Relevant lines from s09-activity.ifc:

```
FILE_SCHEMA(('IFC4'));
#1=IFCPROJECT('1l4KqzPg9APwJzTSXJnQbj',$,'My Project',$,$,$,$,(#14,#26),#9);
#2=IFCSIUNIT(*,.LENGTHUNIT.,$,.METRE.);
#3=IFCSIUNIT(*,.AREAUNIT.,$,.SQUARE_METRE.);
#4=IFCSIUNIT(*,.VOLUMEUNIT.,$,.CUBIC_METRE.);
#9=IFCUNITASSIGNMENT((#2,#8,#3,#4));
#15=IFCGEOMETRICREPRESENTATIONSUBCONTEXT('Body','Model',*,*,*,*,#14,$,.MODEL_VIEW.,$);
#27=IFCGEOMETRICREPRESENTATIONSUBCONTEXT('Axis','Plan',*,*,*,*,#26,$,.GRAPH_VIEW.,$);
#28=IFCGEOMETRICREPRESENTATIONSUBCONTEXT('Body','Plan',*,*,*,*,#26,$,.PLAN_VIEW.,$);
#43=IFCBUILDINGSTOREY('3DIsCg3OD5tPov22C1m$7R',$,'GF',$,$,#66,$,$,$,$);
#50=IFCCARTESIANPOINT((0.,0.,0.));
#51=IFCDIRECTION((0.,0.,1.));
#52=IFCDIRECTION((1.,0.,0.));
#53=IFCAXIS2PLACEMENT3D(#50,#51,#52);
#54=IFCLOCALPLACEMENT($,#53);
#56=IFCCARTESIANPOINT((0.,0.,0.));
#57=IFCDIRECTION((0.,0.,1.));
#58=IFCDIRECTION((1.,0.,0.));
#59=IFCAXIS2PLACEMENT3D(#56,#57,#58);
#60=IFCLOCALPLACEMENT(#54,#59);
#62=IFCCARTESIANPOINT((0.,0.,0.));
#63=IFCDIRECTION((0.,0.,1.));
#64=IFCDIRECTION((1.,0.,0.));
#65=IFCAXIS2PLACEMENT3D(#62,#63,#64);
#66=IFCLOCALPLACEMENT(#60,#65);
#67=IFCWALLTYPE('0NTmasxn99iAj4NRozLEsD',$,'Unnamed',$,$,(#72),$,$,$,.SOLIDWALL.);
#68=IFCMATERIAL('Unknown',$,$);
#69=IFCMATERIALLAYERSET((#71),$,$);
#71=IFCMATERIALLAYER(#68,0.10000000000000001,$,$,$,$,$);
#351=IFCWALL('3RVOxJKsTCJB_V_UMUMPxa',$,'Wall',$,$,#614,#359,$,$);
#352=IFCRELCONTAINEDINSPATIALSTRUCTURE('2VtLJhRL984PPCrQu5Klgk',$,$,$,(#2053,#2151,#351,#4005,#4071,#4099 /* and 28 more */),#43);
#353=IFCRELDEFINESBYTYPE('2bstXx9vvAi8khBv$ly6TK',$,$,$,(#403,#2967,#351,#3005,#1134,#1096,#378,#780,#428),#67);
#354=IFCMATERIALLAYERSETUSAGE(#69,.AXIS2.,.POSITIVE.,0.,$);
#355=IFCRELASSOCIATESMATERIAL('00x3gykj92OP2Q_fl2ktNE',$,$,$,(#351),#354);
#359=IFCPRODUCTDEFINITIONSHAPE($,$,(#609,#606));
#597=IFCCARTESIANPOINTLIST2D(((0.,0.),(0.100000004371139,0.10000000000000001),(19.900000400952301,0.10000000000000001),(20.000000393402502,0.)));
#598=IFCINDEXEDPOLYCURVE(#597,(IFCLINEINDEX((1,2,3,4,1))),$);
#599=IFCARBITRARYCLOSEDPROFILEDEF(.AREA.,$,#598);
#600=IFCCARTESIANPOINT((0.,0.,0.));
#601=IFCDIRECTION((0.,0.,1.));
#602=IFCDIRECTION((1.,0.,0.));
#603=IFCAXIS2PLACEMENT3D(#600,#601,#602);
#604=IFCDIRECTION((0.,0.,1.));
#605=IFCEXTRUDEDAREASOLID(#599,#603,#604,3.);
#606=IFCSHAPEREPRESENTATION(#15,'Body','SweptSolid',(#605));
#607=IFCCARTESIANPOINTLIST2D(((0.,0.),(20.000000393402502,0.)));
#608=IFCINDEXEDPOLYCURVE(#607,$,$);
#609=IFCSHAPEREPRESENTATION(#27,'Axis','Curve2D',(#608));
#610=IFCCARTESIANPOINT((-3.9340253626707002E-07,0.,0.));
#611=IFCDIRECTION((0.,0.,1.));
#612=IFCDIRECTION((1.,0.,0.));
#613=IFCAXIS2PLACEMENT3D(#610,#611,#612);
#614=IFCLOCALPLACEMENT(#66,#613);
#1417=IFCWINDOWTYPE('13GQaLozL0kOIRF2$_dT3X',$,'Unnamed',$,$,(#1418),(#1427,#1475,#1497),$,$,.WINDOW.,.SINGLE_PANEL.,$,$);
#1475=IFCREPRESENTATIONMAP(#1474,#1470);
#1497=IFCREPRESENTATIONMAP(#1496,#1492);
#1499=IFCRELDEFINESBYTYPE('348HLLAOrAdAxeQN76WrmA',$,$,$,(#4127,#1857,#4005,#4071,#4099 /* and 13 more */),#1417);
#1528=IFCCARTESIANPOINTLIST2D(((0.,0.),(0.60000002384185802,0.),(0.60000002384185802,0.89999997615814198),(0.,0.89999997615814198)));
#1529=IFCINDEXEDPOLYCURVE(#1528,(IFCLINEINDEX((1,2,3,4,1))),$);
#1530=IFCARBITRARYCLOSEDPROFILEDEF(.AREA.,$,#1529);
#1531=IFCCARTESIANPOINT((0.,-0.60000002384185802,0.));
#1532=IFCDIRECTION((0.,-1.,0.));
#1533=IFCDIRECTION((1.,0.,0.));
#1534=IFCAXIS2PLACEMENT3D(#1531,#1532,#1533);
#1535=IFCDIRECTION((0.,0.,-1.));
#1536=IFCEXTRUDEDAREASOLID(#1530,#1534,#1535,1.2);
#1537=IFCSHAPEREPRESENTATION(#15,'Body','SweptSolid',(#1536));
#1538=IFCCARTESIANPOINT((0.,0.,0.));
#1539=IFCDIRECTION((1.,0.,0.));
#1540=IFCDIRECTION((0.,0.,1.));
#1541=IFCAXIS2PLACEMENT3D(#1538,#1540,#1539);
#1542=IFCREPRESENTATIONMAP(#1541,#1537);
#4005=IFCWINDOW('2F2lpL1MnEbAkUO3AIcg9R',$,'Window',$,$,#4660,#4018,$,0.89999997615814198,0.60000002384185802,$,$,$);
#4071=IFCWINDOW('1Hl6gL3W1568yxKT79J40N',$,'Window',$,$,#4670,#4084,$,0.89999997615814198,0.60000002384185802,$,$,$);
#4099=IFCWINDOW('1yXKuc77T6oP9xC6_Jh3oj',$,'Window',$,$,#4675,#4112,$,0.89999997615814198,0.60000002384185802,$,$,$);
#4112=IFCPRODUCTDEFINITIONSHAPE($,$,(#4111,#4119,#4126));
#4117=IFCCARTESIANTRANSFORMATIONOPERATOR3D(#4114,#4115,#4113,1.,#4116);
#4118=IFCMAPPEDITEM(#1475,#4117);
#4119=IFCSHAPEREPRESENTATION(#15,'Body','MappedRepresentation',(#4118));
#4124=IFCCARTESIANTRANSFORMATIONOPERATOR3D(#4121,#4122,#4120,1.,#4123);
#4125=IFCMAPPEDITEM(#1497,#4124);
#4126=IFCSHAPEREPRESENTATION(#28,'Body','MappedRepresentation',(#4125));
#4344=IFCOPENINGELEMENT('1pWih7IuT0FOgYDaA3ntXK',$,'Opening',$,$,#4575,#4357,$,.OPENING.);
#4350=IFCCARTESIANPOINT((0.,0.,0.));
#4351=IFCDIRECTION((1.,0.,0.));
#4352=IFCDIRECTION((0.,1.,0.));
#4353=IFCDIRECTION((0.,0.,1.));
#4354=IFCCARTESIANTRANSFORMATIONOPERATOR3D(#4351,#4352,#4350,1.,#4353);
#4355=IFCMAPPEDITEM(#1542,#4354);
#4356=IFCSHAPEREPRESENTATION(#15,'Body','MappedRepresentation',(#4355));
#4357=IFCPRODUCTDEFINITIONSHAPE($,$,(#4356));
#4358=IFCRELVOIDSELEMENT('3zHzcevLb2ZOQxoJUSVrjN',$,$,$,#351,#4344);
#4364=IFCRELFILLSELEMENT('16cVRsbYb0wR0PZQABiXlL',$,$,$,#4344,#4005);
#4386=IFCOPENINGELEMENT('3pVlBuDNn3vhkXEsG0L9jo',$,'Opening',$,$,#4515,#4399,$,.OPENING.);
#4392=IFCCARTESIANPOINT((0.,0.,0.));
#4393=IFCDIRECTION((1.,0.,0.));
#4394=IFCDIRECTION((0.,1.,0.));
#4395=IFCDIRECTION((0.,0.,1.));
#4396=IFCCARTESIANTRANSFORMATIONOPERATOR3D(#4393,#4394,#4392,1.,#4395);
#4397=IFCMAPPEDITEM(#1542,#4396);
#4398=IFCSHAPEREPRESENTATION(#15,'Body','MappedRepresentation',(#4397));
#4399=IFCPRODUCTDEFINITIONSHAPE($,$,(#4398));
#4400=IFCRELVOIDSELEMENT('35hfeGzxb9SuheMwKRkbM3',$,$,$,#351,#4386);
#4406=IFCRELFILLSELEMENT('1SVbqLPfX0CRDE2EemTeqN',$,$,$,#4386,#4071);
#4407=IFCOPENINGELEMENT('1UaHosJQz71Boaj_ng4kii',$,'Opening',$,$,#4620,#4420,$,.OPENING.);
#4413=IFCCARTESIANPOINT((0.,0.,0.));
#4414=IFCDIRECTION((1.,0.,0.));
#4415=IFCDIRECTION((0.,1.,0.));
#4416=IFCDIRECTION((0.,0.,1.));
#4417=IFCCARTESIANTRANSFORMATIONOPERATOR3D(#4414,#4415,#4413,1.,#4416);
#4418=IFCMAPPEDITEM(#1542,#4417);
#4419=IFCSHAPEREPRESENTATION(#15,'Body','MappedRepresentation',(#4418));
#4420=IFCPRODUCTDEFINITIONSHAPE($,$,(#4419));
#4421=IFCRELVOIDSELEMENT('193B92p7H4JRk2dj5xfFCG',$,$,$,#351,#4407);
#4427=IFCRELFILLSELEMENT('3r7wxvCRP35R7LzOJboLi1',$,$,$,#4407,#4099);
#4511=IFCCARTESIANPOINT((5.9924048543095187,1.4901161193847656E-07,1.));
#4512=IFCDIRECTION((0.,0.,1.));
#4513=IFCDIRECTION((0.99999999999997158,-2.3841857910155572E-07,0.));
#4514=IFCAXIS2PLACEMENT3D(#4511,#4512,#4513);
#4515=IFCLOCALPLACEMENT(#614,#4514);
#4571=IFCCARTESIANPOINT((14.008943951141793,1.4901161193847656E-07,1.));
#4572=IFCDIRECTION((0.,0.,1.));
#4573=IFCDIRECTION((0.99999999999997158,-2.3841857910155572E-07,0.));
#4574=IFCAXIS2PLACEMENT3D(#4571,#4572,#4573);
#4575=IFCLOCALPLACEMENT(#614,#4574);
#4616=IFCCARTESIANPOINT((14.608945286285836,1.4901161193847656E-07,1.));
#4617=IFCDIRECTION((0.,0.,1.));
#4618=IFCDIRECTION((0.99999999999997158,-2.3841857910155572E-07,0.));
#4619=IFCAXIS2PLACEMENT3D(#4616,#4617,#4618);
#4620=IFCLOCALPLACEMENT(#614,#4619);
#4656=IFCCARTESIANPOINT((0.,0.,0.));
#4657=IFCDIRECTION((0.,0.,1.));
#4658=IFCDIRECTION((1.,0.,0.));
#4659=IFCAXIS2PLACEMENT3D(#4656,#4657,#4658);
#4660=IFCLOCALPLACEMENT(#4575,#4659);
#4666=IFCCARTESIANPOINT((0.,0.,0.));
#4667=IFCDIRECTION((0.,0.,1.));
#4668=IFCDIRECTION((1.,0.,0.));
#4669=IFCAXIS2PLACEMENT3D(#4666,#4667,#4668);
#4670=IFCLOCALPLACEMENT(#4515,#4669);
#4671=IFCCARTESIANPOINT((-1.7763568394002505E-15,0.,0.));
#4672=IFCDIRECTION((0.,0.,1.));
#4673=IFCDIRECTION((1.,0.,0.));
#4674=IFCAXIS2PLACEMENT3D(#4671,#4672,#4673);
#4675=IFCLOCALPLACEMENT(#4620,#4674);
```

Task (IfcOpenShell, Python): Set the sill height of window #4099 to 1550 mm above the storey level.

```python
import numpy as np
import ifcopenshell
import ifcopenshell.api.geometry
import ifcopenshell.geom
import ifcopenshell.util.element
import ifcopenshell.util.placement
import ifcopenshell.util.shape
import ifcopenshell.util.unit

model = ifcopenshell.open("s09-activity.ifc")
unit_scale = ifcopenshell.util.unit.calculate_unit_scale(model)

window = model.by_id(4099)
opening = window.FillsVoids[0].RelatingOpeningElement
storey = ifcopenshell.util.element.get_container(window, ifc_class="IfcBuildingStorey")
level = ifcopenshell.util.placement.get_local_placement(storey.ObjectPlacement)[2, 3]

# The opening's origin need not be at the sill, so measure its lowest point.
shape = ifcopenshell.geom.create_shape(ifcopenshell.geom.settings(), opening)
bottom = ifcopenshell.util.shape.get_shape_bottom_elevation(shape, shape.geometry) / unit_scale
dz = level + 1.55 - bottom

shift = np.array([0.0, 0.0, dz])
# The window is placed relative to its opening, so it follows when the opening moves.
matrix = ifcopenshell.util.placement.get_local_placement(opening.ObjectPlacement)
matrix[:3, 3] += shift
ifcopenshell.api.geometry.edit_object_placement(
    model, product=opening, matrix=matrix, is_si=False, should_transform_children=True
)

print(f"moved by {dz * unit_scale:+.3f} m")

model.write("s09-activity_v2.ifc")
```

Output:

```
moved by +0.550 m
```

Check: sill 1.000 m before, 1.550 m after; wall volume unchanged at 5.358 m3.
